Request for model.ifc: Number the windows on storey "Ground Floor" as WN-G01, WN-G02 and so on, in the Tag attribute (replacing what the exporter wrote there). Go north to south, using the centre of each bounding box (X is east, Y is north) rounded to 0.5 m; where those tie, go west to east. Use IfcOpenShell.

First a look at what the model holds.

```python
import ifcopenshell
import ifcopenshell.util.element
import ifcopenshell.util.placement

model = ifcopenshell.open("model.ifc")
print(model.schema)
storey = next(s for s in model.by_type("IfcBuildingStorey") if s.Name == "Ground Floor")
windows = [e for e in ifcopenshell.util.element.get_decomposition(storey) if e.is_a("IfcWindow")]
for e in sorted(windows, key=lambda e: e.id()):
    origin = ifcopenshell.util.placement.get_local_placement(e.ObjectPlacement)[:3, 3]
    print(e.id(), e.Tag, e.Name, origin.round(2) + 0.0, sep=" | ")
```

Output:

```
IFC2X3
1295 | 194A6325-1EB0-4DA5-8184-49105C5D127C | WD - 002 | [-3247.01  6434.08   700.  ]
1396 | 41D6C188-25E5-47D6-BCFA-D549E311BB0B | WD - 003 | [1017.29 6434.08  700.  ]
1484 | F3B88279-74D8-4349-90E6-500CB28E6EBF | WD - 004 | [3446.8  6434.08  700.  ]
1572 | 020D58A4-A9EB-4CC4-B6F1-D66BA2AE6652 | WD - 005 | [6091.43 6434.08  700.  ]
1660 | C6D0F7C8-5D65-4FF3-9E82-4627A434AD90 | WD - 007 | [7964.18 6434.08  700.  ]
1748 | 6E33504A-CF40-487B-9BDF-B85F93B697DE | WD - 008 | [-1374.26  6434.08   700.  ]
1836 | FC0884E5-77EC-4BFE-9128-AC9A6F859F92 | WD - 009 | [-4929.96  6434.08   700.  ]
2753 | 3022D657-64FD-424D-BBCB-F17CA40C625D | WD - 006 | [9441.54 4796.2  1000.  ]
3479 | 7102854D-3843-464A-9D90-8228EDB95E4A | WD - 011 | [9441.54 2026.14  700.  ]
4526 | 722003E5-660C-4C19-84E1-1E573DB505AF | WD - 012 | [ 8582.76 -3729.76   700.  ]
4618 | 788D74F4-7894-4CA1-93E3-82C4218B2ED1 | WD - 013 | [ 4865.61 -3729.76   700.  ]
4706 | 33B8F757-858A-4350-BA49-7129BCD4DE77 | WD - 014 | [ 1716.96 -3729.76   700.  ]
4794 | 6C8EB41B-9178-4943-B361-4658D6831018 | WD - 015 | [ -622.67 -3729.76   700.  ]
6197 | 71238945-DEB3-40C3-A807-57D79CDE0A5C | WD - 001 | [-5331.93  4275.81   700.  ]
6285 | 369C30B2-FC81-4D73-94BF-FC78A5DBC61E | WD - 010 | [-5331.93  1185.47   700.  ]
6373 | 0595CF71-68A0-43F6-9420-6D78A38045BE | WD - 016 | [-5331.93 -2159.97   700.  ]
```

```python
import ifcopenshell
import ifcopenshell.geom
import ifcopenshell.util.element
import ifcopenshell.util.shape

model = ifcopenshell.open("model.ifc")
settings = ifcopenshell.geom.settings()
settings.set("use-world-coords", True)


def centre(element):
    shape = ifcopenshell.geom.create_shape(settings, element)
    return ifcopenshell.util.shape.get_bbox_centroid(shape.geometry)


storey = next(s for s in model.by_type("IfcBuildingStorey") if s.Name == "Ground Floor")
windows = [e for e in ifcopenshell.util.element.get_decomposition(storey) if e.is_a("IfcWindow")]

# Insertion points can sit at a corner or the storey origin, so sort by the geometry (in metres).
centres = {e: centre(e) for e in windows}
windows.sort(key=lambda e: (-round(centres[e][1] / 0.5), centres[e][0]))

for i, e in enumerate(windows, start=1):
    number = f"WN-G{i:02d}"
    e.Tag = number
    print(e.id(), number)

model.write("model-out.ifc")
```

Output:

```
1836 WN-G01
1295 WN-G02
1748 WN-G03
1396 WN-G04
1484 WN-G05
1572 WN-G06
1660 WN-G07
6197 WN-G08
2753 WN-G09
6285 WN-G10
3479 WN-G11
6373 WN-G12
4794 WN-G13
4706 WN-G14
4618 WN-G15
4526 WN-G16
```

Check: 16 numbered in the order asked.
